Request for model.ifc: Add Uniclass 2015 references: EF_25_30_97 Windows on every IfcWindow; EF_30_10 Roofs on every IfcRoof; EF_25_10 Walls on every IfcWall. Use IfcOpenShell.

First a look at what the model holds.

```python
import ifcopenshell

model = ifcopenshell.open("model.ifc")
print(model.schema)
print("classifications:", [c.Name for c in model.by_type("IfcClassification")])
for ifc_class in ("IfcDoor", "IfcRoof", "IfcStair", "IfcWall", "IfcWindow"):
    print(ifc_class, len(model.by_type(ifc_class)))
```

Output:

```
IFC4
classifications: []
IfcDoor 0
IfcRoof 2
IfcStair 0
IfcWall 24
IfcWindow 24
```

```python
import ifcopenshell
import ifcopenshell.api.classification

model = ifcopenshell.open("model.ifc")

system = ifcopenshell.api.classification.add_classification(model, classification="Uniclass 2015")

codes = {
    "IfcWindow": ("EF_25_30_97", "Windows"),
    "IfcRoof": ("EF_30_10", "Roofs"),
    "IfcWall": ("EF_25_10", "Walls"),
}
for ifc_class, (code, name) in codes.items():
    products = model.by_type(ifc_class)
    ifcopenshell.api.classification.add_reference(
        model, products=products, classification=system, identification=code, name=name
    )
    print(code, len(products))

model.write("model_v2.ifc")
```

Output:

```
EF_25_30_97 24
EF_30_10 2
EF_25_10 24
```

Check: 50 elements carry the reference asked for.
